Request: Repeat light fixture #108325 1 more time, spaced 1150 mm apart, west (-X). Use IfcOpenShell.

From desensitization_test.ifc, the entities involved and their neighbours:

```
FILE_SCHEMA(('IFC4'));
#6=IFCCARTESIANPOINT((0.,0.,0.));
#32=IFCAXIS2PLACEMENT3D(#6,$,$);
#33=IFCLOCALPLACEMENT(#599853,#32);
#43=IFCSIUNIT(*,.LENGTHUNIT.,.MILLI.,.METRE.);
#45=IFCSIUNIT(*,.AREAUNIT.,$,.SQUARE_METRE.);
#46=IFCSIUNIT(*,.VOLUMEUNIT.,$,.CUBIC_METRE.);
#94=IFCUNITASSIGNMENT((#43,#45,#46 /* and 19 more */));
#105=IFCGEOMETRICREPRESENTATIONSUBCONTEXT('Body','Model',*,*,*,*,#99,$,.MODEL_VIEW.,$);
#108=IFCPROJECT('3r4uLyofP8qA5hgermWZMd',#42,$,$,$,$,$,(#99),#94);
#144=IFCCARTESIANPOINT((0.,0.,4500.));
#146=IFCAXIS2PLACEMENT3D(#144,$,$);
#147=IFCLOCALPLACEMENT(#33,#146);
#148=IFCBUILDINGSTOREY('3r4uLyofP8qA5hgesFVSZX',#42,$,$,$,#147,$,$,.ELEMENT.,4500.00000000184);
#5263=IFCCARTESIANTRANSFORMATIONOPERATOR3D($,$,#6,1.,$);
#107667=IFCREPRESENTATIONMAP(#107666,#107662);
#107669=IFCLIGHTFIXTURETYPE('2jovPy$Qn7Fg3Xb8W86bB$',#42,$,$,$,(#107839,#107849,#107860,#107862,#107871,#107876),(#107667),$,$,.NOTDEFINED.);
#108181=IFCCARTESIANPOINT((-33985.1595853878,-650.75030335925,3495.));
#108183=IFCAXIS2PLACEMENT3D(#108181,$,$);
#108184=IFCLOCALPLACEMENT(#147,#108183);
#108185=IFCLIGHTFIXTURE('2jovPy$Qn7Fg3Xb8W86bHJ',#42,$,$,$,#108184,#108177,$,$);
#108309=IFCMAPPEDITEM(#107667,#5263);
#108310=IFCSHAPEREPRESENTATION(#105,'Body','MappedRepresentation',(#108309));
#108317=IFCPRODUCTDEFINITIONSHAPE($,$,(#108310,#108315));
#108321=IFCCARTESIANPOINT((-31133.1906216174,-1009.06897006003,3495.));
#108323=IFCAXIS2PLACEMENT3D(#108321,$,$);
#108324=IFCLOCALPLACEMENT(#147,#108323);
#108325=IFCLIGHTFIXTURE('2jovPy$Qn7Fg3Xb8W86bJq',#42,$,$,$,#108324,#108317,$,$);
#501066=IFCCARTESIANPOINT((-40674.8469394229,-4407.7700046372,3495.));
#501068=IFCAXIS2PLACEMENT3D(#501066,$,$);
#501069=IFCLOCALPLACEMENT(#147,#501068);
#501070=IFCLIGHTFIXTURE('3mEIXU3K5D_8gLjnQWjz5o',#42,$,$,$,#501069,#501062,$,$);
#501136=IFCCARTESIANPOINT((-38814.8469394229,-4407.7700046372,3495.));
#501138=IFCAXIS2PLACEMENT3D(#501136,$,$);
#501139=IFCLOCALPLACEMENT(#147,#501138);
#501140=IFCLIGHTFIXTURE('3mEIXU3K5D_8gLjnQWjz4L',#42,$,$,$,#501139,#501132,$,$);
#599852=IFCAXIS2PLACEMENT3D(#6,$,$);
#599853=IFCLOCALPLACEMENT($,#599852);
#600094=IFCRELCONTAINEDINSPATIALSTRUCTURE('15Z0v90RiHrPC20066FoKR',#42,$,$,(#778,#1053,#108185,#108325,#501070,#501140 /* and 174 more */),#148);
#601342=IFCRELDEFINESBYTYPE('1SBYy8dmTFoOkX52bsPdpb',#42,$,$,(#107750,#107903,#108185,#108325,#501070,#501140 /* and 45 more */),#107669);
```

```python
import numpy as np
import ifcopenshell
import ifcopenshell.api.geometry
import ifcopenshell.api.root
import ifcopenshell.util.element
import ifcopenshell.util.placement

model = ifcopenshell.open("desensitization_test.ifc")


def reuse_history(source, copy):
    """copy_class also copies each property set's owner history, people and application; keep the originals."""
    for rel in copy.IsDefinedBy:
        if rel.is_a("IfcRelDefinesByProperties") and (history := rel.RelatingPropertyDefinition.OwnerHistory):
            rel.RelatingPropertyDefinition.OwnerHistory = source.OwnerHistory
            ifcopenshell.util.element.remove_deep2(model, history)


source = model.by_guid("2jovPy$Qn7Fg3Xb8W86bJq")
base = ifcopenshell.util.placement.get_local_placement(source.ObjectPlacement)
step = np.array([-1.0, 0.0, 0.0]) * 1150.0

for i in range(1, 2):
    copy = ifcopenshell.api.root.copy_class(model, product=source)
    copy.Representation = ifcopenshell.util.element.copy_deep(
        model, source.Representation, exclude=["IfcGeometricRepresentationContext", "IfcRepresentationMap"]
    )
    reuse_history(source, copy)
    matrix = base.copy()
    matrix[:3, 3] += i * step
    print("added at", matrix[:3, 3].round(3) + 0.0)
    ifcopenshell.api.geometry.edit_object_placement(model, product=copy, matrix=matrix, is_si=False)

model.write("desensitization_test_updated.ifc")
```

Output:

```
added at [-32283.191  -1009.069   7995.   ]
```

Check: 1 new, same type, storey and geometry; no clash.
